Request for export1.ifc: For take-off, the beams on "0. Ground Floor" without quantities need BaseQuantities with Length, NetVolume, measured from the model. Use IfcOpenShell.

First a look at what the model holds.

```python
import ifcopenshell
import ifcopenshell.util.element
import ifcopenshell.util.unit

model = ifcopenshell.open("export1.ifc")
print(model.schema)
for unit_type in ("LENGTHUNIT", "AREAUNIT", "VOLUMEUNIT"):
    print(unit_type, ifcopenshell.util.unit.calculate_unit_scale(model, unit_type))
storey = next(s for s in model.by_type("IfcBuildingStorey") if s.Name == "0. Ground Floor")
beams = [e for e in ifcopenshell.util.element.get_decomposition(storey) if e.is_a("IfcBeam")]
for e in sorted(beams, key=lambda e: e.id()):
    print(e.id(), e.is_a(), e.Name, list(ifcopenshell.util.element.get_psets(e, qtos_only=True)), sep=" | ")
```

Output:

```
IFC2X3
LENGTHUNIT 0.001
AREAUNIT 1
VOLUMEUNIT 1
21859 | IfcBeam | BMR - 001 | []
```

```python
import ifcopenshell
import ifcopenshell.api.pset
import ifcopenshell.geom
import ifcopenshell.util.element
import ifcopenshell.util.shape
import ifcopenshell.util.unit

model = ifcopenshell.open("export1.ifc")
unit_scale = ifcopenshell.util.unit.calculate_unit_scale(model)
volume_scale = ifcopenshell.util.unit.calculate_unit_scale(model, "VOLUMEUNIT")
settings = ifcopenshell.geom.settings()

storey = next(s for s in model.by_type("IfcBuildingStorey") if s.Name == "0. Ground Floor")
beams = [e for e in ifcopenshell.util.element.get_decomposition(storey) if e.is_a("IfcBeam")]

for e in sorted(beams, key=lambda e: e.id()):
    if ifcopenshell.util.element.get_psets(e, qtos_only=True, should_inherit=False):
        continue
    # Geometry comes back in metres, in the element's own axes.
    shape = ifcopenshell.geom.create_shape(settings, e)
    values = {
        "Length": ifcopenshell.util.shape.get_max_xyz(shape.geometry) / unit_scale,
        "NetVolume": ifcopenshell.util.shape.get_volume(shape.geometry) / volume_scale,
    }
    qto = ifcopenshell.api.pset.add_qto(model, product=e, name="BaseQuantities")
    ifcopenshell.api.pset.edit_qto(model, qto=qto, properties=values)
    print(e.id(), {k: round(v, 3) for k, v in values.items()})

model.write("export1_updated.ifc")
```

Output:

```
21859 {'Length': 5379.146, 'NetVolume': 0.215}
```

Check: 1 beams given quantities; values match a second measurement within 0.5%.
